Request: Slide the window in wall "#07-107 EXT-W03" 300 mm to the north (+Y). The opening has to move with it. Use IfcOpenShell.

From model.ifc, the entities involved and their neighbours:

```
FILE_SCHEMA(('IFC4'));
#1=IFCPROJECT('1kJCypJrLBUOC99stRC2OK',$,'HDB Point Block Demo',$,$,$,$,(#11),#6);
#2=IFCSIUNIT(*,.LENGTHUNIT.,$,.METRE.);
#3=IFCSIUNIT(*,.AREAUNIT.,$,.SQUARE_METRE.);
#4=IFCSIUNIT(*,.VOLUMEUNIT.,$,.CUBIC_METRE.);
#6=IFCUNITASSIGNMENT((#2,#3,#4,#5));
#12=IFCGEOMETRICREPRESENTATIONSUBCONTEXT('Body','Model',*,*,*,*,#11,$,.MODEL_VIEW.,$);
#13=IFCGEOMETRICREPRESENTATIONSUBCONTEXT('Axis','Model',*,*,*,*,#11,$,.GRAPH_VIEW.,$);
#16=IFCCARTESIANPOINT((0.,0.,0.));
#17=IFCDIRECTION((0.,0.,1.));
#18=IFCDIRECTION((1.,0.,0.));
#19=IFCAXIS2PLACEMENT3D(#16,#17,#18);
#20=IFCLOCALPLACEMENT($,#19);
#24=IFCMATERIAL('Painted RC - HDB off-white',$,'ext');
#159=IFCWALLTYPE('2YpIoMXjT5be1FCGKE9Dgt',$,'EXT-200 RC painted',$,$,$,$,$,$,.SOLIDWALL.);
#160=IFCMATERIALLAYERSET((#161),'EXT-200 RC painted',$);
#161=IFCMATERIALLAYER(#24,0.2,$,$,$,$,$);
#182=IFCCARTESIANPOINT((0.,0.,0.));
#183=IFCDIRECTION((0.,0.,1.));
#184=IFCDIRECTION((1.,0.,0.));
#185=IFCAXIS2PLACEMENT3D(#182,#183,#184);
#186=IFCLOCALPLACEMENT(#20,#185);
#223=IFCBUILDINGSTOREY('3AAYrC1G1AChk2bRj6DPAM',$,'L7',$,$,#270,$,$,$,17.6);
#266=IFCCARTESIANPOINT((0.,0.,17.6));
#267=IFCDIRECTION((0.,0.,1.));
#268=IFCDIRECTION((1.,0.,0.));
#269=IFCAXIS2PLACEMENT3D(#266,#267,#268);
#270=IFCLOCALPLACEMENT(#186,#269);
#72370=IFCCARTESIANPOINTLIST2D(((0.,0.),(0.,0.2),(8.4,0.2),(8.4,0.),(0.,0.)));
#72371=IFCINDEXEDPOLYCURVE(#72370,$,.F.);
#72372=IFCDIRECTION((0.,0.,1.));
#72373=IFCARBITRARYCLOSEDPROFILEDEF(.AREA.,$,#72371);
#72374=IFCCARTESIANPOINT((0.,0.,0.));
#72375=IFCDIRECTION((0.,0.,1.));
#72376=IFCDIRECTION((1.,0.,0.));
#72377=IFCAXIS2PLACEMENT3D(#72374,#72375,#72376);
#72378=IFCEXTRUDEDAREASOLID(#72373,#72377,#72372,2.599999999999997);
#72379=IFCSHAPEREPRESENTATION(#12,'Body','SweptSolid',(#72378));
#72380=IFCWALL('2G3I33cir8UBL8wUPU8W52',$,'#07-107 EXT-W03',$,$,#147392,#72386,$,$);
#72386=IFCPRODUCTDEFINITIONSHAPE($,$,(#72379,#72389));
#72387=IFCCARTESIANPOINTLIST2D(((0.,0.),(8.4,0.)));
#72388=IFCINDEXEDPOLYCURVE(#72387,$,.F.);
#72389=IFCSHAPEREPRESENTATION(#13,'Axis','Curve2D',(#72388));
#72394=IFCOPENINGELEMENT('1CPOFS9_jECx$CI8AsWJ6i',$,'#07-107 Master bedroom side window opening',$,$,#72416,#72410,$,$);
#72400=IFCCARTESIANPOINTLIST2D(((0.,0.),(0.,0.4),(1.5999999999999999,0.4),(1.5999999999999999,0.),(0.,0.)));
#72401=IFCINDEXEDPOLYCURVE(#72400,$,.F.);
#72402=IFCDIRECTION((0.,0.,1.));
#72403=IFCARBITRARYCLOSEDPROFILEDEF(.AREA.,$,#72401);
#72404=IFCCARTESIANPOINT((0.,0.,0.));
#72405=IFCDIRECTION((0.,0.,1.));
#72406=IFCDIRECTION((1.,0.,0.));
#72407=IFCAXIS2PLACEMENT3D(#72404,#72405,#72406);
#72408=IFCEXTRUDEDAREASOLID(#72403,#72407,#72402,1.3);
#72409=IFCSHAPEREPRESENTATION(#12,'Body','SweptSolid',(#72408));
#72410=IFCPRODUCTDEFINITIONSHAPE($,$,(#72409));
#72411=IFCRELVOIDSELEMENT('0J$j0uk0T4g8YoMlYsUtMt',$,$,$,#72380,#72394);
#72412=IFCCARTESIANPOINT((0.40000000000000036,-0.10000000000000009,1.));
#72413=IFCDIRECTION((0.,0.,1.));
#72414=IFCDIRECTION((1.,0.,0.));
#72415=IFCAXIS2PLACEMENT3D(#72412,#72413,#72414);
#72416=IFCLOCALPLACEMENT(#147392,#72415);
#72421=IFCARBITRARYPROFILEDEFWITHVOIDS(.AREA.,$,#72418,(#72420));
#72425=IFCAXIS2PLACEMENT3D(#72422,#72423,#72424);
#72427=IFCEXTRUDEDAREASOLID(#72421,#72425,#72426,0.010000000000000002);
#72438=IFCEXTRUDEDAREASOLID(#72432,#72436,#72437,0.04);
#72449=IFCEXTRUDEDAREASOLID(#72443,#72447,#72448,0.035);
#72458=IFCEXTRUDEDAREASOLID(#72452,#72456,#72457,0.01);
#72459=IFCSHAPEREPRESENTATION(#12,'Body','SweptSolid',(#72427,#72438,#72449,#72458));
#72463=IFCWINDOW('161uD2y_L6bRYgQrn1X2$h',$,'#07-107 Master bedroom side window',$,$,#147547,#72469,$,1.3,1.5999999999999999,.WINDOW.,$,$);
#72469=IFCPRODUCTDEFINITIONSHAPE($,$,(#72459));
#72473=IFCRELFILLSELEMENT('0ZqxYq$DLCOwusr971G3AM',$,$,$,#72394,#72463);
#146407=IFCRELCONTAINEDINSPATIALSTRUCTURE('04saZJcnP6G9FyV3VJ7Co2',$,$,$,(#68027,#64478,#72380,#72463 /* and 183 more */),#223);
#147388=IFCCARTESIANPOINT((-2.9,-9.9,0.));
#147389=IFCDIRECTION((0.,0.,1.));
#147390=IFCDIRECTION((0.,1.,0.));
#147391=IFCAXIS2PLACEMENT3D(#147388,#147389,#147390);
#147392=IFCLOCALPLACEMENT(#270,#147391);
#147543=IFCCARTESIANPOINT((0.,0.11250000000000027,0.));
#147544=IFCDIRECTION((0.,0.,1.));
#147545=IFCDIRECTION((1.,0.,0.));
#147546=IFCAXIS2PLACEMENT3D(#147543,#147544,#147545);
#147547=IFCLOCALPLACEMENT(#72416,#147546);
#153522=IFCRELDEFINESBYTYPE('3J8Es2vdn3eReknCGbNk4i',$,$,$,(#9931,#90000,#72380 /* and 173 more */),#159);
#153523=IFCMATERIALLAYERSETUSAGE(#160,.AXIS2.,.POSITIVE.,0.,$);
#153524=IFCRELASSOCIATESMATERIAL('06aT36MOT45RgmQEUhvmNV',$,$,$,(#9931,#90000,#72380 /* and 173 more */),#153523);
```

```python
import ifcopenshell
import ifcopenshell.api.geometry
import ifcopenshell.util.placement
import ifcopenshell.util.unit

model = ifcopenshell.open("model.ifc")
unit_scale = ifcopenshell.util.unit.calculate_unit_scale(model)

window = model.by_id(72463)
opening = window.FillsVoids[0].RelatingOpeningElement
wall = opening.VoidsElements[0].RelatingBuildingElement

wall_matrix = ifcopenshell.util.placement.get_local_placement(wall.ObjectPlacement)
shift = wall_matrix[:3, 0] * 0.3 / unit_scale
before = ifcopenshell.util.placement.get_local_placement(window.ObjectPlacement)[:3, 3].copy()

# The window is placed relative to its opening, so it follows when the opening moves.
matrix = ifcopenshell.util.placement.get_local_placement(opening.ObjectPlacement)
matrix[:3, 3] += shift
ifcopenshell.api.geometry.edit_object_placement(
    model, product=opening, matrix=matrix, is_si=False, should_transform_children=True
)

after = ifcopenshell.util.placement.get_local_placement(window.ObjectPlacement)[:3, 3]
print("window moved by", (after - before).round(3) + 0.0)

model.write("model_edited.ifc")
```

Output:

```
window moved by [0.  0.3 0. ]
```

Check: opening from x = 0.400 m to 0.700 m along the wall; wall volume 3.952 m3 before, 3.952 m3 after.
